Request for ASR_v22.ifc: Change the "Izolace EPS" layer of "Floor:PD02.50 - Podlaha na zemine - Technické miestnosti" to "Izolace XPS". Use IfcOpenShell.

First a look at what the model holds.

```python
import ifcopenshell
import ifcopenshell.util.element

model = ifcopenshell.open("ASR_v22.ifc")
print(model.schema)
for layer_set in model.by_type("IfcMaterialLayerSet"):
    if layer_set.LayerSetName == "Floor:PD02.50 - Podlaha na zemine - Technické miestnosti":
        for layer in layer_set.MaterialLayers:
            print(layer.id(), layer.Material and layer.Material.Name, layer.LayerThickness, sep=" | ")
        print(len(ifcopenshell.util.element.get_elements_by_material(model, layer_set)), "elements and types use it")
print(sorted(m.Name for m in model.by_type("IfcMaterial") if m.Name)[:60])
```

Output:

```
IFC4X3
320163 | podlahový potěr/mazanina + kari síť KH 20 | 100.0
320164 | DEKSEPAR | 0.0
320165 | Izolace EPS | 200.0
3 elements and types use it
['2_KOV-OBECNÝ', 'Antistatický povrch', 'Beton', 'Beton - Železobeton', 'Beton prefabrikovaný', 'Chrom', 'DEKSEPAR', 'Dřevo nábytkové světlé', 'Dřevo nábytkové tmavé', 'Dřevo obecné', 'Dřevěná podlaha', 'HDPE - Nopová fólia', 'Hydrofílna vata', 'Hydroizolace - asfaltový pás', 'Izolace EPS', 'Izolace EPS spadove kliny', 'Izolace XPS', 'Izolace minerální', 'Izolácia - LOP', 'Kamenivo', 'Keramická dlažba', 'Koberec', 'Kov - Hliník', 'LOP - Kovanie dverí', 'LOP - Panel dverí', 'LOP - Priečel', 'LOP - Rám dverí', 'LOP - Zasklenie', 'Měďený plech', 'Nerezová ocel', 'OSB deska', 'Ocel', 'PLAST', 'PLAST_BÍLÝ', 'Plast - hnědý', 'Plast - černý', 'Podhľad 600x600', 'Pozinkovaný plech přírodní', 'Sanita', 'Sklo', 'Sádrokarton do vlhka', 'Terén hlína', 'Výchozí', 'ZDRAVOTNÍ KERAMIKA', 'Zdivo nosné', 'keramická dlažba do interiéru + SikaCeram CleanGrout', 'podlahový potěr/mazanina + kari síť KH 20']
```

```python
import ifcopenshell
import ifcopenshell.api.material

model = ifcopenshell.open("ASR_v22.ifc")

layer_set = next(s for s in model.by_type("IfcMaterialLayerSet") if s.LayerSetName == "Floor:PD02.50 - Podlaha na zemine - Technické miestnosti")
layer = next(l for l in layer_set.MaterialLayers if l.Material and l.Material.Name == "Izolace EPS")
material = next(m for m in model.by_type("IfcMaterial") if m.Name == "Izolace XPS")

# Point this one layer at the other material; renaming the old one would change it everywhere.
ifcopenshell.api.material.edit_layer(model, layer=layer, attributes={"Name": material.Name}, material=material)

print([l.Material.Name if l.Material else None for l in layer_set.MaterialLayers])

model.write("ASR_v22-out.ifc")
```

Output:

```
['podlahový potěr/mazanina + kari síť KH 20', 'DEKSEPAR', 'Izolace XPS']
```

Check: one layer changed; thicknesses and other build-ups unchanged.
